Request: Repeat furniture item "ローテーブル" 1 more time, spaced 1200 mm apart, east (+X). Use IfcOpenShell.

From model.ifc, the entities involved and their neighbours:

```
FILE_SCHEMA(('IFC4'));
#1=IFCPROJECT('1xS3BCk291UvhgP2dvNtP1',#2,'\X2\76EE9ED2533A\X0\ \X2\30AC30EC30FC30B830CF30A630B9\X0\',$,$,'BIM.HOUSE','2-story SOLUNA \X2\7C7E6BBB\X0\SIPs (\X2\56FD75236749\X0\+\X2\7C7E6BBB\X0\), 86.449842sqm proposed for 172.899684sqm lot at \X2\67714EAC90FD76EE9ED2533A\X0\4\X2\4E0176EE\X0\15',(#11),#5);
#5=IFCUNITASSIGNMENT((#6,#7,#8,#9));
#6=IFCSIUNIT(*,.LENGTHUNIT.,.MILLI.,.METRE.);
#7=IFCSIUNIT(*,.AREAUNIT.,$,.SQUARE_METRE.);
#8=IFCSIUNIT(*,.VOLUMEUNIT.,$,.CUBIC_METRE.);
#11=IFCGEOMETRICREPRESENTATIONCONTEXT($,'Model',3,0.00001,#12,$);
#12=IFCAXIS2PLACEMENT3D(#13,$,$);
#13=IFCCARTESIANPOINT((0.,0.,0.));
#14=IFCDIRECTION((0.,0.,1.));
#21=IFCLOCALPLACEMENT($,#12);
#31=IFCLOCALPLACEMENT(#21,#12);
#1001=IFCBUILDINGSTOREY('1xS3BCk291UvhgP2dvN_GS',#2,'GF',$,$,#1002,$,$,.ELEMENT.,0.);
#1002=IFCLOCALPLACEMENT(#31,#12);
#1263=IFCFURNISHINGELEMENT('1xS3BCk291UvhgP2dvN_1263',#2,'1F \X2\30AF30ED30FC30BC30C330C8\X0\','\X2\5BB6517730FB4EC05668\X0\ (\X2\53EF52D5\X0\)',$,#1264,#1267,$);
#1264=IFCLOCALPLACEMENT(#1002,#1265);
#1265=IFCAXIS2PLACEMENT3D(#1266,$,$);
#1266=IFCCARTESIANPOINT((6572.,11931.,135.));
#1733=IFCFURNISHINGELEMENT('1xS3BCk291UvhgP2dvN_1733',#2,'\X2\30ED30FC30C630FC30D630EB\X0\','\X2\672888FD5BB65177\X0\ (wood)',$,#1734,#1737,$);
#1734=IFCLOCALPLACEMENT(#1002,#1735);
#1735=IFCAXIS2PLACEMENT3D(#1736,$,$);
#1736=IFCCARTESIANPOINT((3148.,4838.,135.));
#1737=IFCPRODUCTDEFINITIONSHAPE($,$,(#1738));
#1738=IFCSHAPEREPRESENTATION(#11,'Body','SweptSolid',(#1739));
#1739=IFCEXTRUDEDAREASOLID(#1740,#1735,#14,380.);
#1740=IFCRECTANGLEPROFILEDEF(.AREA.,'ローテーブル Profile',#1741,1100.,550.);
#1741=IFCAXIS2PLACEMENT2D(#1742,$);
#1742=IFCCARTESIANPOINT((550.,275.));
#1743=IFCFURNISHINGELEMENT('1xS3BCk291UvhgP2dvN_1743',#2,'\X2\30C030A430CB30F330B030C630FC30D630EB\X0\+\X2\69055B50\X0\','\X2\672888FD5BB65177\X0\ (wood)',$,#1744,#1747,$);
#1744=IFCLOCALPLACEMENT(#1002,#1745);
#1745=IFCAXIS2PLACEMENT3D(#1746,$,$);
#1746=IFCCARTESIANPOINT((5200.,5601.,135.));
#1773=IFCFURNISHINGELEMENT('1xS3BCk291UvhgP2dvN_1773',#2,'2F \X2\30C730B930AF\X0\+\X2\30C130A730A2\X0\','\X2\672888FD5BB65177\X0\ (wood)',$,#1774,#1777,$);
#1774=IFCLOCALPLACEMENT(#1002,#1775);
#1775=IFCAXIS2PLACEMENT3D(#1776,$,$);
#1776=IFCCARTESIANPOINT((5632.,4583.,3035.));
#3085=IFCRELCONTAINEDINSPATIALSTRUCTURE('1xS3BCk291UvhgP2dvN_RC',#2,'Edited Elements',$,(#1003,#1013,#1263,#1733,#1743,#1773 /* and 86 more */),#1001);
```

```python
import numpy as np
import ifcopenshell
import ifcopenshell.api.geometry
import ifcopenshell.api.root
import ifcopenshell.util.element
import ifcopenshell.util.placement
import ifcopenshell.util.unit

model = ifcopenshell.open("model.ifc")
unit_scale = ifcopenshell.util.unit.calculate_unit_scale(model)


def reuse_history(source, copy):
    """copy_class also copies each property set's owner history, people and application; keep the originals."""
    for rel in copy.IsDefinedBy:
        if rel.is_a("IfcRelDefinesByProperties") and (history := rel.RelatingPropertyDefinition.OwnerHistory):
            rel.RelatingPropertyDefinition.OwnerHistory = source.OwnerHistory
            ifcopenshell.util.element.remove_deep2(model, history)


source = model.by_guid("1xS3BCk291UvhgP2dvN_1733")
base = ifcopenshell.util.placement.get_local_placement(source.ObjectPlacement)
step = np.array([1.0, 0.0, 0.0]) * 1.2 / unit_scale

for i in range(1, 2):
    copy = ifcopenshell.api.root.copy_class(model, product=source)
    copy.Representation = ifcopenshell.util.element.copy_deep(
        model, source.Representation, exclude=["IfcGeometricRepresentationContext", "IfcRepresentationMap"]
    )
    reuse_history(source, copy)
    matrix = base.copy()
    matrix[:3, 3] += i * step
    print("added at", matrix[:3, 3].round(3) + 0.0)
    ifcopenshell.api.geometry.edit_object_placement(model, product=copy, matrix=matrix, is_si=False)

model.write("model_updated.ifc")
```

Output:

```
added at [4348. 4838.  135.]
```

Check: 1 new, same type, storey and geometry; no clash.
